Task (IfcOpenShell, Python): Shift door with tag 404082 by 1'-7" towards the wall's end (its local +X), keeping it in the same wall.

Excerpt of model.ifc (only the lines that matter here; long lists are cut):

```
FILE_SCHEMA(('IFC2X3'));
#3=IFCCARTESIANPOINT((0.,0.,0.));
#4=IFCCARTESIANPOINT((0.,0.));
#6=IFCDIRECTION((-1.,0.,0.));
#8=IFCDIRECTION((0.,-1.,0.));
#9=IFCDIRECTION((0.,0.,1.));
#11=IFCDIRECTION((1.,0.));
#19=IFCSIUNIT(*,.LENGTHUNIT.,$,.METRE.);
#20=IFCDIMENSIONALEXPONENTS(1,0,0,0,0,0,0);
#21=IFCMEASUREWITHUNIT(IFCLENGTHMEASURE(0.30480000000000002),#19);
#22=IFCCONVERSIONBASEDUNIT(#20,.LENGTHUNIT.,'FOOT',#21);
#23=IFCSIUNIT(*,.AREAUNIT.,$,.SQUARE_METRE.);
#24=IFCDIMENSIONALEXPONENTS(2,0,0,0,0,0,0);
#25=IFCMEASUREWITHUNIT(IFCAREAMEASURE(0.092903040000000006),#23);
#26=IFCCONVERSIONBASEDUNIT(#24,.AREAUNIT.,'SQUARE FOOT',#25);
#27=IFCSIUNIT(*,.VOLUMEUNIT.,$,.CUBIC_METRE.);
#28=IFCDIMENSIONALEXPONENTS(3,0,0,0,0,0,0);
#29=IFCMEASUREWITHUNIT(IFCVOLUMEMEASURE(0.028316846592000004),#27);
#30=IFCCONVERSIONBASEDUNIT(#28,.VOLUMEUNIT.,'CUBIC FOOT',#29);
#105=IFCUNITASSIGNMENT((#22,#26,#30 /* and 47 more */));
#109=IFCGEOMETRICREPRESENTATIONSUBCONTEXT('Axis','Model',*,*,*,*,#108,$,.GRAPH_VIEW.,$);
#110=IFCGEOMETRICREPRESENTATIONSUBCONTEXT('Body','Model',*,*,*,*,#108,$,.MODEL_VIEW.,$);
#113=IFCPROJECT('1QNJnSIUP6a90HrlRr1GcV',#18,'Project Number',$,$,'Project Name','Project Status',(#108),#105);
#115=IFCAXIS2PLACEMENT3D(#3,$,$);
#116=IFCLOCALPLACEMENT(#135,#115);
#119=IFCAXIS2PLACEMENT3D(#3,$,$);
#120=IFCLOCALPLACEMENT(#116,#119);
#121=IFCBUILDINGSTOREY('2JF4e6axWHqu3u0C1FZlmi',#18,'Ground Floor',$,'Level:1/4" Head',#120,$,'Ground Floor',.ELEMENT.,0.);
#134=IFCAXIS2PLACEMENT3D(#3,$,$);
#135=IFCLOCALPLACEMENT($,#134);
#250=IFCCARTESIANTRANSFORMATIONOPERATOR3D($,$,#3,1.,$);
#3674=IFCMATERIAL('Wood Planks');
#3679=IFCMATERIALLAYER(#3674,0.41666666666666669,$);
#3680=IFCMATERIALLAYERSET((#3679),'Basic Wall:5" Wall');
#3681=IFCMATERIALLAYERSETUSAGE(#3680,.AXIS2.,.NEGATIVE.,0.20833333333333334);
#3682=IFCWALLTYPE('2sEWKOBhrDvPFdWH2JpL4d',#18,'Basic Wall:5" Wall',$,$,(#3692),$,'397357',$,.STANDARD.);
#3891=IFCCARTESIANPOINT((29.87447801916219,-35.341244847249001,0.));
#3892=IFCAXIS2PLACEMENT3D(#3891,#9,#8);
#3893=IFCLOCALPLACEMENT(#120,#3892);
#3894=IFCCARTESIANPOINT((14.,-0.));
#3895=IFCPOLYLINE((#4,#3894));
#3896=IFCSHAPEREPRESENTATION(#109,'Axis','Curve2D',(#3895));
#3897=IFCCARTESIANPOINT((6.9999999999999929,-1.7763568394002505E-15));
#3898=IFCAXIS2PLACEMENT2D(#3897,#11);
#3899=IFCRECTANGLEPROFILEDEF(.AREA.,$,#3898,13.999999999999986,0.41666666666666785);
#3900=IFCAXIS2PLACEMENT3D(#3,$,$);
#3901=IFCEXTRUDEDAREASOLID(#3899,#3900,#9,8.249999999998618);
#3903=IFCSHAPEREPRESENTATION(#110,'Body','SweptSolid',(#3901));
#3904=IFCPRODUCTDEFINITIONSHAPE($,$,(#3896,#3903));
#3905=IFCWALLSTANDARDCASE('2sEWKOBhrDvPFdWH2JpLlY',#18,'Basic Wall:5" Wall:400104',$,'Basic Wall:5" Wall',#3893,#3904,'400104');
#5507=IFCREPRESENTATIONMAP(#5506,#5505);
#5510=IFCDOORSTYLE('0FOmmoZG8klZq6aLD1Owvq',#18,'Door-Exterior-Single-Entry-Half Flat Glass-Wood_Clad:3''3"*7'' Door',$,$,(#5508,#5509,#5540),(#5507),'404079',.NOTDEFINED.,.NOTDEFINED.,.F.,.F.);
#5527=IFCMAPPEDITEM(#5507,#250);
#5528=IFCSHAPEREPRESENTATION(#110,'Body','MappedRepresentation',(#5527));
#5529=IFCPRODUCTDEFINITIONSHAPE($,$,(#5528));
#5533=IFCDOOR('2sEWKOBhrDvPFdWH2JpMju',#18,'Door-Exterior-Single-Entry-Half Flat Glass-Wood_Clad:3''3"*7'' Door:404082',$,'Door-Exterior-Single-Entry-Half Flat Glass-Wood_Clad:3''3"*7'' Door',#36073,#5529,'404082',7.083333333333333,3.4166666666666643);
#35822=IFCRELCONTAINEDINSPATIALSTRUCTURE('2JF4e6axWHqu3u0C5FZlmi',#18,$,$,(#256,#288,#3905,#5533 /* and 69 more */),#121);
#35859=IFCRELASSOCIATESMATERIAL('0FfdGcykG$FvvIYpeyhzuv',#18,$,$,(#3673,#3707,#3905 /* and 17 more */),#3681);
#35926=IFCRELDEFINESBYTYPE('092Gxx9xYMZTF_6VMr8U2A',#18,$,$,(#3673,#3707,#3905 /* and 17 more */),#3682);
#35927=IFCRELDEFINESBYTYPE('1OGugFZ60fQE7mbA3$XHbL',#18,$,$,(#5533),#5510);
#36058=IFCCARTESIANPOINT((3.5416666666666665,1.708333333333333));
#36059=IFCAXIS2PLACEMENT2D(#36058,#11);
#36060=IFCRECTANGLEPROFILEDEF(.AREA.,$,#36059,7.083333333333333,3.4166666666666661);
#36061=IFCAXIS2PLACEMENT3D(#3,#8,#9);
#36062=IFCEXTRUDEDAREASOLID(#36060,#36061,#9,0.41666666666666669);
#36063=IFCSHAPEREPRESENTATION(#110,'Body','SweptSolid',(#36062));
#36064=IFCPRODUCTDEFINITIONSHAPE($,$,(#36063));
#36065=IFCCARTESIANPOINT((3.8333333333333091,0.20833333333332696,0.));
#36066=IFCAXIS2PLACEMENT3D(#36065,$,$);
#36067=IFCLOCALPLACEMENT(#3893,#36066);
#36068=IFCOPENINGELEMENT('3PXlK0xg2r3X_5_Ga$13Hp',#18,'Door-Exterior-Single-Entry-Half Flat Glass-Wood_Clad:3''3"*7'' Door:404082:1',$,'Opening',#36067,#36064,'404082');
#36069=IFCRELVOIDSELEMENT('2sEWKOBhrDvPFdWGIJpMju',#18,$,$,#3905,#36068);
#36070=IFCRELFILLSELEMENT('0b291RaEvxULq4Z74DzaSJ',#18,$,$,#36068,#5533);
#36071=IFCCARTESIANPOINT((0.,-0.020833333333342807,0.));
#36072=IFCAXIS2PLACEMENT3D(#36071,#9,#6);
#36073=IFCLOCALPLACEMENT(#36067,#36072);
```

```python
import ifcopenshell
import ifcopenshell.api.geometry
import ifcopenshell.util.placement
import ifcopenshell.util.unit

model = ifcopenshell.open("model.ifc")
unit_scale = ifcopenshell.util.unit.calculate_unit_scale(model)

door = model.by_id(5533)
opening = door.FillsVoids[0].RelatingOpeningElement
wall = opening.VoidsElements[0].RelatingBuildingElement

wall_matrix = ifcopenshell.util.placement.get_local_placement(wall.ObjectPlacement)
shift = wall_matrix[:3, 0] * 19 * 0.0254 / unit_scale
before = ifcopenshell.util.placement.get_local_placement(door.ObjectPlacement)[:3, 3].copy()

# The door is placed relative to its opening, so it follows when the opening moves.
matrix = ifcopenshell.util.placement.get_local_placement(opening.ObjectPlacement)
matrix[:3, 3] += shift
ifcopenshell.api.geometry.edit_object_placement(
    model, product=opening, matrix=matrix, is_si=False, should_transform_children=True
)

after = ifcopenshell.util.placement.get_local_placement(door.ObjectPlacement)[:3, 3]
print("door moved by", (after - before).round(3) + 0.0)

model.write("model_rev.ifc")
```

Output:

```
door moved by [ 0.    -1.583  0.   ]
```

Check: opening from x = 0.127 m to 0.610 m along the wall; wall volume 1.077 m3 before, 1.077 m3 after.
